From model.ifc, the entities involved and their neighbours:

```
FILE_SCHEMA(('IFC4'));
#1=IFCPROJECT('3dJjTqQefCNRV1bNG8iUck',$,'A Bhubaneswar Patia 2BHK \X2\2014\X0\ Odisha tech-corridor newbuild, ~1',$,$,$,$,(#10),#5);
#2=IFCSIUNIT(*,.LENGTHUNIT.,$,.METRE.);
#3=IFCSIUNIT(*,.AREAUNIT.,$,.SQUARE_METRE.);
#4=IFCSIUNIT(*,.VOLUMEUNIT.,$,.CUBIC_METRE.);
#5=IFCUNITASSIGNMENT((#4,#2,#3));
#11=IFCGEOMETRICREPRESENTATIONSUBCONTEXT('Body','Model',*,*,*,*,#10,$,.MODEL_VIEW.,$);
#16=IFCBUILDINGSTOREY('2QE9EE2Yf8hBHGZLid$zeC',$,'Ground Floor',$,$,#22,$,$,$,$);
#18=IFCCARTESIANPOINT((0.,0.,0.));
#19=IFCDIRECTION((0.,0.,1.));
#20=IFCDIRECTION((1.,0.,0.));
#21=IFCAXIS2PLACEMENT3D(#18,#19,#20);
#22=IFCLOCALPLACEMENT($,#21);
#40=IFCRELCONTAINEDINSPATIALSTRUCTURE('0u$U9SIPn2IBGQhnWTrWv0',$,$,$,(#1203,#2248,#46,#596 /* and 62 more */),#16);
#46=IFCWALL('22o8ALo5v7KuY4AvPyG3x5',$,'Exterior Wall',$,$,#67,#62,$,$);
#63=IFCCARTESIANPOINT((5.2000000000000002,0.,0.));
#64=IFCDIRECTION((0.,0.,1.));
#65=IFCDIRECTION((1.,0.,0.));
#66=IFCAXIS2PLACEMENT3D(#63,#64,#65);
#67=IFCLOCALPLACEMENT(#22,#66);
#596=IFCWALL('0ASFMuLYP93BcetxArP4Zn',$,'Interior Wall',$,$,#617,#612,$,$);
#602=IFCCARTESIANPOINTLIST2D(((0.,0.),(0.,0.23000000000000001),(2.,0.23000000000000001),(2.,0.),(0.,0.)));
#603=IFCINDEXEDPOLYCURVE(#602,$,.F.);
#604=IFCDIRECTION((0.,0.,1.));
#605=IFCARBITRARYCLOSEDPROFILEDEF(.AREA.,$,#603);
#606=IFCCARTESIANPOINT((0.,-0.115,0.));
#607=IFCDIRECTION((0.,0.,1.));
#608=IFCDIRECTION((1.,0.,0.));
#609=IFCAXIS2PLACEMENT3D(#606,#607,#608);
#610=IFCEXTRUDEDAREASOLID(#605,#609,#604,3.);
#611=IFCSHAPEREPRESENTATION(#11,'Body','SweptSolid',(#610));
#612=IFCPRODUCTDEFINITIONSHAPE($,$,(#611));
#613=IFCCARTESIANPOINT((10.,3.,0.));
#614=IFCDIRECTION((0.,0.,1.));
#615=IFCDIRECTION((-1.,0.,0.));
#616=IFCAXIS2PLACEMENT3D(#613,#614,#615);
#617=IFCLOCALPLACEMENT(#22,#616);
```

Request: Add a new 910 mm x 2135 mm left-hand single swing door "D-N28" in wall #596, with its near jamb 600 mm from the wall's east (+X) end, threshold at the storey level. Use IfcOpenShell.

```python
import numpy as np
import ifcopenshell
import ifcopenshell.api.feature
import ifcopenshell.api.geometry
import ifcopenshell.api.root
import ifcopenshell.api.spatial
import ifcopenshell.geom
import ifcopenshell.util.element
import ifcopenshell.util.placement
import ifcopenshell.util.representation
import ifcopenshell.util.shape
import ifcopenshell.util.unit

model = ifcopenshell.open("model.ifc")
unit_scale = ifcopenshell.util.unit.calculate_unit_scale(model)
settings = ifcopenshell.geom.settings()


def volume(element):
    """Net volume in cubic metres, openings subtracted."""
    shape = ifcopenshell.geom.create_shape(settings, element)
    return ifcopenshell.util.shape.get_volume(shape.geometry)


wall = model.by_id(596)
storey = ifcopenshell.util.element.get_container(wall, ifc_class="IfcBuildingStorey")
context = ifcopenshell.util.representation.get_context(model, "Model", "Body", "MODEL_VIEW")
before = volume(wall)

width, height, from_end, sill = 0.91, 2.135, 0.6, 0.0  # metres

# The wall runs along its own X axis, and the end named is its -X end.
wall_shape = ifcopenshell.geom.create_shape(settings, wall)
x, y, z = ifcopenshell.util.shape.get_vertices(wall_shape.geometry).T
start = x.min() + from_end
face, thickness = float(y.min()), float(y.max() - y.min())
wall_matrix = ifcopenshell.util.placement.get_local_placement(wall.ObjectPlacement)
level = ifcopenshell.util.placement.get_local_placement(storey.ObjectPlacement)[2, 3]


def in_wall(x, y):
    """Placement at x, y metres in the wall's axes, at sill height."""
    matrix = wall_matrix.copy()
    matrix[:, 3] = wall_matrix @ np.array([x / unit_scale, y / unit_scale, 0.0, 1.0])
    matrix[2, 3] = level + sill / unit_scale
    return matrix


# Opening: a box that overshoots both wall faces by 50 mm.
opening = ifcopenshell.api.root.create_entity(model, ifc_class="IfcOpeningElement", predefined_type="OPENING")
box = ifcopenshell.api.geometry.add_wall_representation(
    model, context=context, length=width, height=height, thickness=thickness + 0.1
)
ifcopenshell.api.geometry.assign_representation(model, product=opening, representation=box)
ifcopenshell.api.geometry.edit_object_placement(model, product=opening, matrix=in_wall(start, face - 0.05), is_si=False)
ifcopenshell.api.feature.add_feature(model, feature=opening, element=wall)

door = ifcopenshell.api.root.create_entity(model, ifc_class="IfcDoor", name="D-N28", predefined_type="DOOR")
door.OverallWidth, door.OverallHeight = width / unit_scale, height / unit_scale
door.OperationType = "SINGLE_SWING_LEFT"
body = ifcopenshell.api.geometry.add_door_representation(
    model,
    context=context,
    overall_width=door.OverallWidth,
    overall_height=door.OverallHeight,
    operation_type="SINGLE_SWING_LEFT",
    lining_properties={"LiningDepth": thickness / unit_scale, "ThresholdDepth": thickness / unit_scale},
)
ifcopenshell.api.geometry.assign_representation(model, product=door, representation=body)
ifcopenshell.api.spatial.assign_container(model, products=[door], relating_structure=storey)
ifcopenshell.api.feature.add_filling(model, opening=opening, element=door)

# The lining spans the wall, so the door starts at the wall face.
ifcopenshell.api.geometry.edit_object_placement(model, product=door, matrix=in_wall(start, face), is_si=False)

after = volume(wall)

print(f"wall volume {before:.3f} -> {after:.3f} m3")

model.write("model-out.ifc")
```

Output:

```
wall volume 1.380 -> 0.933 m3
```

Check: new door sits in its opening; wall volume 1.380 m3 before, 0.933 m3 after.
